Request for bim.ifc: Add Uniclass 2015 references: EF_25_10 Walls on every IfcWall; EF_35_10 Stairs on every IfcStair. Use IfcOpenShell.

First a look at what the model holds.

```python
import ifcopenshell

model = ifcopenshell.open("bim.ifc")
print(model.schema)
print("classifications:", [c.Name for c in model.by_type("IfcClassification")])
for ifc_class in ("IfcDoor", "IfcRoof", "IfcStair", "IfcWall", "IfcWindow"):
    print(ifc_class, len(model.by_type(ifc_class)))
```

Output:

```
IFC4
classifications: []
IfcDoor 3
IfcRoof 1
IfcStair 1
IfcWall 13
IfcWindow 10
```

```python
import ifcopenshell
import ifcopenshell.api.classification

model = ifcopenshell.open("bim.ifc")

system = ifcopenshell.api.classification.add_classification(model, classification="Uniclass 2015")

codes = {
    "IfcWall": ("EF_25_10", "Walls"),
    "IfcStair": ("EF_35_10", "Stairs"),
}
for ifc_class, (code, name) in codes.items():
    products = model.by_type(ifc_class)
    ifcopenshell.api.classification.add_reference(
        model, products=products, classification=system, identification=code, name=name
    )
    print(code, len(products))

model.write("bim_v2.ifc")
```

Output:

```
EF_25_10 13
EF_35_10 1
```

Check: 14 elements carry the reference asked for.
